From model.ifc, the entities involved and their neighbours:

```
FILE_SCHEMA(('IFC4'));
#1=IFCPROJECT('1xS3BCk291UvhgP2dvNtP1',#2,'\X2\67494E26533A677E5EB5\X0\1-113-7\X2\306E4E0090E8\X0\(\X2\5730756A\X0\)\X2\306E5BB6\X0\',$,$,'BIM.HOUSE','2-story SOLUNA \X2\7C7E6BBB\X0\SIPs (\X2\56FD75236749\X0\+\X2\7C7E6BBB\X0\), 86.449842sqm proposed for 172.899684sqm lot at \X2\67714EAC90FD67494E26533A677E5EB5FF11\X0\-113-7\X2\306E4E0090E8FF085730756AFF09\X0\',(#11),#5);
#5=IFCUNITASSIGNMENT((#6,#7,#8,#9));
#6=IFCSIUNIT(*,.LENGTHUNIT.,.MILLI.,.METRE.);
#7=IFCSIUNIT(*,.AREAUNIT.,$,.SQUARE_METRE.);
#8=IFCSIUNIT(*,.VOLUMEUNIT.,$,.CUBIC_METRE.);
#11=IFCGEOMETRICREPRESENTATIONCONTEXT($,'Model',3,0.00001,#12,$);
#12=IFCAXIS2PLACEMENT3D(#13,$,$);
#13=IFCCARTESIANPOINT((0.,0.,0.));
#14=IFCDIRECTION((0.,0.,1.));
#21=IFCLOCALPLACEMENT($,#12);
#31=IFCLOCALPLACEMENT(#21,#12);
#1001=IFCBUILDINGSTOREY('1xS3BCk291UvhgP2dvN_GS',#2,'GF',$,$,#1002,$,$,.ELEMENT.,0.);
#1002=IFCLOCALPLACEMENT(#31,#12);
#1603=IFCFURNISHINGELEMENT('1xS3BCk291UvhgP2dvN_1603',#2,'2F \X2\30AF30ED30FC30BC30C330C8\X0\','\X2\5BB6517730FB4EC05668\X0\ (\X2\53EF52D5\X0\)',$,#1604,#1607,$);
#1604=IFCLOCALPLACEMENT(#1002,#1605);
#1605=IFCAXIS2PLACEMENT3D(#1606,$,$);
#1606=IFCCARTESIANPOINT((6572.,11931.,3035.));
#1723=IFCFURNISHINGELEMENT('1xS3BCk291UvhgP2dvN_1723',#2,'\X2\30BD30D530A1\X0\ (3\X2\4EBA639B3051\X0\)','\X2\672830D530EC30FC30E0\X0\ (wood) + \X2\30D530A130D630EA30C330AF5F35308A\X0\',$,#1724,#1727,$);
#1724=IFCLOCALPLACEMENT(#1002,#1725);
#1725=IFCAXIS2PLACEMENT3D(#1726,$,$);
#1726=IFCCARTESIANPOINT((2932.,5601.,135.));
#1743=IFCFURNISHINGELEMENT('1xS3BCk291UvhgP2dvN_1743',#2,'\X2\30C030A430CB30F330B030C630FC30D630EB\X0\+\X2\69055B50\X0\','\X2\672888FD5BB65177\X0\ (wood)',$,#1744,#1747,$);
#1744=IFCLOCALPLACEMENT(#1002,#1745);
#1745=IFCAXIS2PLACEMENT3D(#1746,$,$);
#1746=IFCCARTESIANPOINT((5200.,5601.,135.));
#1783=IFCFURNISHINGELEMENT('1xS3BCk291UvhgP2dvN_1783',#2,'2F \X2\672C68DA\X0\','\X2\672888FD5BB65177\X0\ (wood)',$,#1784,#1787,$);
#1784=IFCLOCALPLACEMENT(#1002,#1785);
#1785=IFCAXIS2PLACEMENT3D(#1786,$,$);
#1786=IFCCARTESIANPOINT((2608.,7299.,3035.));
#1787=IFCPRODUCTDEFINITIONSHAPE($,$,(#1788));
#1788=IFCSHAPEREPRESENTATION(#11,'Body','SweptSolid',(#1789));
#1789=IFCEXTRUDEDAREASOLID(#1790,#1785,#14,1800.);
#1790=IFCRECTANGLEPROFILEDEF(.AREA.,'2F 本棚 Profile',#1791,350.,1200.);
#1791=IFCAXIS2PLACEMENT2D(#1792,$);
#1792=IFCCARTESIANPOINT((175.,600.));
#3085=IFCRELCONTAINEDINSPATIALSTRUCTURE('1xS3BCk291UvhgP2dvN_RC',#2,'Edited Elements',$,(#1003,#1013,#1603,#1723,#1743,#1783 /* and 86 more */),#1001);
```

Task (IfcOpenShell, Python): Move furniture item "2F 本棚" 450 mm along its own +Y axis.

```python
import ifcopenshell
import ifcopenshell.api.geometry
import ifcopenshell.util.placement

model = ifcopenshell.open("model.ifc")

item = model.by_guid("1xS3BCk291UvhgP2dvN_1783")
matrix = ifcopenshell.util.placement.get_local_placement(item.ObjectPlacement)
matrix[:3, 3] += matrix[:3, 1] * 450.0
ifcopenshell.api.geometry.edit_object_placement(model, product=item, matrix=matrix, is_si=False)

print(ifcopenshell.util.placement.get_local_placement(item.ObjectPlacement).round(3) + 0.0)

model.write("model_rev.ifc")
```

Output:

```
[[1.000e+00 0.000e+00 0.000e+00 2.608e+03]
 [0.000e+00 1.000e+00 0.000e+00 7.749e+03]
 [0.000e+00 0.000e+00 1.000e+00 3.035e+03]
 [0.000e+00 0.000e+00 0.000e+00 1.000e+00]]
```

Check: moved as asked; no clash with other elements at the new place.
